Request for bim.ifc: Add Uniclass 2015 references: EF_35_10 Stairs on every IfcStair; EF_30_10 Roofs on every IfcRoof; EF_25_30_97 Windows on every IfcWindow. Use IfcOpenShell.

First a look at what the model holds.

```python
import ifcopenshell

model = ifcopenshell.open("bim.ifc")
print(model.schema)
print("classifications:", [c.Name for c in model.by_type("IfcClassification")])
for ifc_class in ("IfcDoor", "IfcRoof", "IfcStair", "IfcWall", "IfcWindow"):
    print(ifc_class, len(model.by_type(ifc_class)))
```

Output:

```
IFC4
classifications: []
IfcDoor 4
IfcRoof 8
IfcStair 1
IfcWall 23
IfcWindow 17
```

```python
import ifcopenshell
import ifcopenshell.api.classification

model = ifcopenshell.open("bim.ifc")

system = ifcopenshell.api.classification.add_classification(model, classification="Uniclass 2015")

codes = {
    "IfcStair": ("EF_35_10", "Stairs"),
    "IfcRoof": ("EF_30_10", "Roofs"),
    "IfcWindow": ("EF_25_30_97", "Windows"),
}
for ifc_class, (code, name) in codes.items():
    products = model.by_type(ifc_class)
    ifcopenshell.api.classification.add_reference(
        model, products=products, classification=system, identification=code, name=name
    )
    print(code, len(products))

model.write("bim-out.ifc")
```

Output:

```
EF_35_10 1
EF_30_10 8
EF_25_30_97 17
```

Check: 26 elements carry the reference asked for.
